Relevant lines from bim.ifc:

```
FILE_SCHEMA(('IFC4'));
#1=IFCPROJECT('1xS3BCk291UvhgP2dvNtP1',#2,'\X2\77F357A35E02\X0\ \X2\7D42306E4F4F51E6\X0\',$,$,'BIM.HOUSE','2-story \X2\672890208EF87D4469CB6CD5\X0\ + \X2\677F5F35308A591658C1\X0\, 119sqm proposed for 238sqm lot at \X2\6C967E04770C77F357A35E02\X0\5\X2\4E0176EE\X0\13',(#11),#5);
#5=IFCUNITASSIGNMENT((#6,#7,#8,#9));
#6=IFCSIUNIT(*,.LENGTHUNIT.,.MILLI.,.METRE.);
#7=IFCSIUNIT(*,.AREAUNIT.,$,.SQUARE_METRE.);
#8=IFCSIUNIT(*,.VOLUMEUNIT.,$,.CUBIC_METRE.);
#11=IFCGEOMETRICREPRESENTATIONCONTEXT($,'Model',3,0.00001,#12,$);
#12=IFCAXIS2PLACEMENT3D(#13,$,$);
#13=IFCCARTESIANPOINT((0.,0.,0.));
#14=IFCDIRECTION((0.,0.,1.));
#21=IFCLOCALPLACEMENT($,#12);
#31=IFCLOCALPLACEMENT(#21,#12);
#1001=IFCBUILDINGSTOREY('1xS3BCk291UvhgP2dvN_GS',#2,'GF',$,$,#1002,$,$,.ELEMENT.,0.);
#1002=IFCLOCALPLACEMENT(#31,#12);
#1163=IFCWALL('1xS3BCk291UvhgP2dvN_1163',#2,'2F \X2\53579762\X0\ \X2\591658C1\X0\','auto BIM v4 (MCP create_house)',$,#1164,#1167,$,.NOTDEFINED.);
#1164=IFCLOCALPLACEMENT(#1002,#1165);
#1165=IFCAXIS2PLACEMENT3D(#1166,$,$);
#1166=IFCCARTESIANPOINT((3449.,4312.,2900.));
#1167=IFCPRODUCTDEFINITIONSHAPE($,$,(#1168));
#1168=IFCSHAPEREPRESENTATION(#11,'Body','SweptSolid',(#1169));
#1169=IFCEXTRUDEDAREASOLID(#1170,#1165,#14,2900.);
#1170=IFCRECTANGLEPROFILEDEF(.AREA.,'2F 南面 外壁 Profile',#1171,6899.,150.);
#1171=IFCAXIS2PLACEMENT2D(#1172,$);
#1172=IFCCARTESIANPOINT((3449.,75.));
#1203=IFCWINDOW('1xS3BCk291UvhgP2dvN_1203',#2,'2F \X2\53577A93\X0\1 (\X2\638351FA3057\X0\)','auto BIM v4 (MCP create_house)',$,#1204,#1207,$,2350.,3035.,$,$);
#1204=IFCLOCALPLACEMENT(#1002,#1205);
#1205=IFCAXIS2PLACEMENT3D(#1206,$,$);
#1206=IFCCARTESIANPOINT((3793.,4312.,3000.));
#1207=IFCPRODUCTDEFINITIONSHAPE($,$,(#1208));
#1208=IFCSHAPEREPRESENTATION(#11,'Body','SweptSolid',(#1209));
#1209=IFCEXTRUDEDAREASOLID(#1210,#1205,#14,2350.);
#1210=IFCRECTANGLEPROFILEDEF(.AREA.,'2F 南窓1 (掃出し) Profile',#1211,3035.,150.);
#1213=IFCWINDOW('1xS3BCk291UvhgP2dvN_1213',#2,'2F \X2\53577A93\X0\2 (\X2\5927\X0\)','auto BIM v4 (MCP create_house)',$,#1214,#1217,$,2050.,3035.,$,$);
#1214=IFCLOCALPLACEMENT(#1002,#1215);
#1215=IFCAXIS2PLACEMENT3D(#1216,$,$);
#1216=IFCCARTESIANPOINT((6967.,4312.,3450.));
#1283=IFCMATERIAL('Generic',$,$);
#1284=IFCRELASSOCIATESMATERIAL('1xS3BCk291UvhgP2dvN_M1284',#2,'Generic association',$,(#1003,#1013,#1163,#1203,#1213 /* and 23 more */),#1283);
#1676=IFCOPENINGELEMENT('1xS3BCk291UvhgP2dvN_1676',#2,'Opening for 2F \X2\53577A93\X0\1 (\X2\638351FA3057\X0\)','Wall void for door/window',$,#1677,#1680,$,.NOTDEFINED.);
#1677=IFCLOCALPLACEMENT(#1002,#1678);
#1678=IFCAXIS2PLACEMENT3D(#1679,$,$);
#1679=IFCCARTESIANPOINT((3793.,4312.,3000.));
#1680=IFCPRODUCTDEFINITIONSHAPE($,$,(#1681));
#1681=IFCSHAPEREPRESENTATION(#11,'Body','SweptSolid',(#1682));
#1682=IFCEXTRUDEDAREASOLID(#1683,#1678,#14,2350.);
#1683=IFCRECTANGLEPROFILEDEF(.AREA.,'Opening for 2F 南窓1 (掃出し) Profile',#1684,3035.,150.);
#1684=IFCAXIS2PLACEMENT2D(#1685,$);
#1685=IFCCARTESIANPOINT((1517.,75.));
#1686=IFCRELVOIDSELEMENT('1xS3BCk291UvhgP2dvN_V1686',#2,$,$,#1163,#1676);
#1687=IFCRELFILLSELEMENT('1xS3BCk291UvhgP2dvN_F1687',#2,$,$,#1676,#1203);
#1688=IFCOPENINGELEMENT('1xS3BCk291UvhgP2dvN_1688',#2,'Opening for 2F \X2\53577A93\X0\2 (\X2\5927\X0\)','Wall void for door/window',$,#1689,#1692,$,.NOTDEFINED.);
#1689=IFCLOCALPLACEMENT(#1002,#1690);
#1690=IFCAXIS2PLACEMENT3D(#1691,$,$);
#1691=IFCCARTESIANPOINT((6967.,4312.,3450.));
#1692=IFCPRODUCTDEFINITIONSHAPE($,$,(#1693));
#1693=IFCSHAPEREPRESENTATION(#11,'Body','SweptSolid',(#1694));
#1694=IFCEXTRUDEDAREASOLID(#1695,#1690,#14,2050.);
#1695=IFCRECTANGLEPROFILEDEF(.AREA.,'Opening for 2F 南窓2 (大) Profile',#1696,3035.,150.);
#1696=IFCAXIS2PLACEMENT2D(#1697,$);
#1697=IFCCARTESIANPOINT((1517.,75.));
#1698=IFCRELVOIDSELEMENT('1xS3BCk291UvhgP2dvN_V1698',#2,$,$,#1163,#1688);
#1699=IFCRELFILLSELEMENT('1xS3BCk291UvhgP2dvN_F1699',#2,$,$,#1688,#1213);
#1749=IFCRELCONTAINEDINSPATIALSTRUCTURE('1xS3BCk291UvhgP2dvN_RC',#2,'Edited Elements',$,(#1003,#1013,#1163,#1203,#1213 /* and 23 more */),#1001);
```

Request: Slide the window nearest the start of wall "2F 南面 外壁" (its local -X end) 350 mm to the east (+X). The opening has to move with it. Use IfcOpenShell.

```python
import ifcopenshell
import ifcopenshell.api.geometry
import ifcopenshell.util.placement
import ifcopenshell.util.unit

model = ifcopenshell.open("bim.ifc")
unit_scale = ifcopenshell.util.unit.calculate_unit_scale(model)

window = model.by_id(1203)
opening = window.FillsVoids[0].RelatingOpeningElement
wall = opening.VoidsElements[0].RelatingBuildingElement

wall_matrix = ifcopenshell.util.placement.get_local_placement(wall.ObjectPlacement)
shift = wall_matrix[:3, 0] * 0.35 / unit_scale
before = ifcopenshell.util.placement.get_local_placement(window.ObjectPlacement)[:3, 3].copy()

# The window is not placed relative to its opening, so move both.
for product in (opening, window):
    matrix = ifcopenshell.util.placement.get_local_placement(product.ObjectPlacement)
    matrix[:3, 3] += shift
    ifcopenshell.api.geometry.edit_object_placement(model, product=product, matrix=matrix, is_si=False)

after = ifcopenshell.util.placement.get_local_placement(window.ObjectPlacement)[:3, 3]
print("window moved by", (after - before).round(3) + 0.0)

model.write("bim_v2.ifc")
```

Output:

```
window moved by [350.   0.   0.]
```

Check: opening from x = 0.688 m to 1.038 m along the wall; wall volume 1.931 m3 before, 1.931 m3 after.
